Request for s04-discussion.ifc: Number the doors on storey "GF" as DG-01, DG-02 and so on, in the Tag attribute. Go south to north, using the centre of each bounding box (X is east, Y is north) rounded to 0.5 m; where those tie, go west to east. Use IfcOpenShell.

First a look at what the model holds.

```python
import ifcopenshell
import ifcopenshell.util.element
import ifcopenshell.util.placement

model = ifcopenshell.open("s04-discussion.ifc")
print(model.schema)
storey = next(s for s in model.by_type("IfcBuildingStorey") if s.Name == "GF")
doors = [e for e in ifcopenshell.util.element.get_decomposition(storey) if e.is_a("IfcDoor")]
for e in sorted(doors, key=lambda e: e.id()):
    origin = ifcopenshell.util.placement.get_local_placement(e.ObjectPlacement)[:3, 3]
    print(e.id(), e.Tag, e.Name, origin.round(2) + 0.0, sep=" | ")
```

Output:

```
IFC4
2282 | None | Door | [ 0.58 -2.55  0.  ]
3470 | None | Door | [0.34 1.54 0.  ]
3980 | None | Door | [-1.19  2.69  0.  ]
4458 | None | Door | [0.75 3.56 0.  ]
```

```python
import ifcopenshell
import ifcopenshell.geom
import ifcopenshell.util.element
import ifcopenshell.util.shape

model = ifcopenshell.open("s04-discussion.ifc")
settings = ifcopenshell.geom.settings()
settings.set("use-world-coords", True)


def centre(element):
    shape = ifcopenshell.geom.create_shape(settings, element)
    return ifcopenshell.util.shape.get_bbox_centroid(shape.geometry)


storey = next(s for s in model.by_type("IfcBuildingStorey") if s.Name == "GF")
doors = [e for e in ifcopenshell.util.element.get_decomposition(storey) if e.is_a("IfcDoor")]

# Insertion points can sit at a corner or the storey origin, so sort by the geometry (in metres).
centres = {e: centre(e) for e in doors}
doors.sort(key=lambda e: (round(centres[e][1] / 0.5), centres[e][0]))

for i, e in enumerate(doors, start=1):
    number = f"DG-{i:02d}"
    e.Tag = number
    print(e.id(), number)

model.write("s04-discussion_rev.ifc")
```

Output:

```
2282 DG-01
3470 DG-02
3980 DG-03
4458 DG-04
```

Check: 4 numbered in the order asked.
